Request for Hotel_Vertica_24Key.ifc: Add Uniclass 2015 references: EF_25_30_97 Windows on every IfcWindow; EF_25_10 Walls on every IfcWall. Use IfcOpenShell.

First a look at what the model holds.

```python
import ifcopenshell

model = ifcopenshell.open("Hotel_Vertica_24Key.ifc")
print(model.schema)
print("classifications:", [c.Name for c in model.by_type("IfcClassification")])
for ifc_class in ("IfcDoor", "IfcRoof", "IfcStair", "IfcWall", "IfcWindow"):
    print(ifc_class, len(model.by_type(ifc_class)))
```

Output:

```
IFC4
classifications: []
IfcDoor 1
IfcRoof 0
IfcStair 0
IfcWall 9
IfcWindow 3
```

```python
import ifcopenshell
import ifcopenshell.api.classification

model = ifcopenshell.open("Hotel_Vertica_24Key.ifc")

system = ifcopenshell.api.classification.add_classification(model, classification="Uniclass 2015")

codes = {
    "IfcWindow": ("EF_25_30_97", "Windows"),
    "IfcWall": ("EF_25_10", "Walls"),
}
for ifc_class, (code, name) in codes.items():
    products = model.by_type(ifc_class)
    ifcopenshell.api.classification.add_reference(
        model, products=products, classification=system, identification=code, name=name
    )
    print(code, len(products))

model.write("Hotel_Vertica_24Key_rev.ifc")
```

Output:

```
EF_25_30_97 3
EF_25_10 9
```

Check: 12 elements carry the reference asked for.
